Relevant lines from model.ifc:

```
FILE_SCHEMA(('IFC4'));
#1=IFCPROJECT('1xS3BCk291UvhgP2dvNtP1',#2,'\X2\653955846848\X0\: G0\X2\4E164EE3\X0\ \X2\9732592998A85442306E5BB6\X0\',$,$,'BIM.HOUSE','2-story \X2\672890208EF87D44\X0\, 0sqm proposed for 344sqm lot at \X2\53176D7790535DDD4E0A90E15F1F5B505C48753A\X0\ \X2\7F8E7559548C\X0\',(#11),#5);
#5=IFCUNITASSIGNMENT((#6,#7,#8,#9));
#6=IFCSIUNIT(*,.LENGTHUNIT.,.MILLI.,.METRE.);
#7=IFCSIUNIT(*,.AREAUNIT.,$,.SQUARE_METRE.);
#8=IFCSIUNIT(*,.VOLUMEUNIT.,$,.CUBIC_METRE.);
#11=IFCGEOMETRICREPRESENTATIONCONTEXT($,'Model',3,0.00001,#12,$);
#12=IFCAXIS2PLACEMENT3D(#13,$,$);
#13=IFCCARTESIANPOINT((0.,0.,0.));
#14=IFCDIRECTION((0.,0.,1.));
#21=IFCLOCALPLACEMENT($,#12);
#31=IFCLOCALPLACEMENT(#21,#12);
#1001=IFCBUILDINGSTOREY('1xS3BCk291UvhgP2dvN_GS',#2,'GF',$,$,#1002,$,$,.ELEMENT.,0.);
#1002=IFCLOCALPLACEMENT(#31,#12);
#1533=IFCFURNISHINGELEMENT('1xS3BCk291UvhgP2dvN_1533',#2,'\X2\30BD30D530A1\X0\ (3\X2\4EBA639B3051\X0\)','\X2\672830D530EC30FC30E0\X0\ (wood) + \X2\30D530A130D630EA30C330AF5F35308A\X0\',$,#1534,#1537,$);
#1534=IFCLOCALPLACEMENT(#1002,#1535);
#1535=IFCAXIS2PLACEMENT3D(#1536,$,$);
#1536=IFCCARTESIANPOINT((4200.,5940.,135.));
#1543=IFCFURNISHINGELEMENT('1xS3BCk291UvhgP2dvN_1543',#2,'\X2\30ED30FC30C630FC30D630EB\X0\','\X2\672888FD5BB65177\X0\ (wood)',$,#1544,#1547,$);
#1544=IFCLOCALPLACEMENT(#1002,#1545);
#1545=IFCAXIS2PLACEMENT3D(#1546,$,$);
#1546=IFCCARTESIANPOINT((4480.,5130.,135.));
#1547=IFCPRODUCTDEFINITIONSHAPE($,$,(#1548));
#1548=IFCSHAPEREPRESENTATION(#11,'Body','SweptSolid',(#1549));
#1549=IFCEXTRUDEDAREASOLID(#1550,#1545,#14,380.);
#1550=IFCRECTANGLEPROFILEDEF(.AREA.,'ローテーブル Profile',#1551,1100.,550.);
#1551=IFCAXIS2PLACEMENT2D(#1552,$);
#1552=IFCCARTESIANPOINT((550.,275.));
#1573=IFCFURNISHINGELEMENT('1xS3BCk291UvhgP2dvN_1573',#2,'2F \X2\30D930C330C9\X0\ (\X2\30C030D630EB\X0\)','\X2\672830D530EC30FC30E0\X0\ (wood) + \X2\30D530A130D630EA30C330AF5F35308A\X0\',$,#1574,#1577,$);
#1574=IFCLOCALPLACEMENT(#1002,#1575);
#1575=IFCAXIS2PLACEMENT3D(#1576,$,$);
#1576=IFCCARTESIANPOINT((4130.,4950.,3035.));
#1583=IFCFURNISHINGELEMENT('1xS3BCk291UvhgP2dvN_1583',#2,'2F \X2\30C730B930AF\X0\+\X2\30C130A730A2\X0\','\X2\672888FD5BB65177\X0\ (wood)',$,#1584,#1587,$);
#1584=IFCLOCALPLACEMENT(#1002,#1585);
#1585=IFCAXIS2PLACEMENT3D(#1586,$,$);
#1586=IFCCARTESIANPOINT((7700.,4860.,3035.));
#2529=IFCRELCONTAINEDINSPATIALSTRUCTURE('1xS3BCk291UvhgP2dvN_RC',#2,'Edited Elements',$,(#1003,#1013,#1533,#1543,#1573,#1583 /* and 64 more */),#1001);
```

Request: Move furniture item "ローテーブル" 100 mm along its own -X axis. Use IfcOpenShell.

```python
import ifcopenshell
import ifcopenshell.api.geometry
import ifcopenshell.util.placement
import ifcopenshell.util.unit

model = ifcopenshell.open("model.ifc")
unit_scale = ifcopenshell.util.unit.calculate_unit_scale(model)

item = model.by_guid("1xS3BCk291UvhgP2dvN_1543")
matrix = ifcopenshell.util.placement.get_local_placement(item.ObjectPlacement)
matrix[:3, 3] -= matrix[:3, 0] * 0.1 / unit_scale
ifcopenshell.api.geometry.edit_object_placement(model, product=item, matrix=matrix, is_si=False)

print(ifcopenshell.util.placement.get_local_placement(item.ObjectPlacement).round(3) + 0.0)

model.write("model-out.ifc")
```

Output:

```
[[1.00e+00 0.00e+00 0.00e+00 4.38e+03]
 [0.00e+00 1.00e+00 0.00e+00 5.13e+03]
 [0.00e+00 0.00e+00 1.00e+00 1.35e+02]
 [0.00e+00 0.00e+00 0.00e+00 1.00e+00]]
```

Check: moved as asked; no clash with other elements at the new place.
